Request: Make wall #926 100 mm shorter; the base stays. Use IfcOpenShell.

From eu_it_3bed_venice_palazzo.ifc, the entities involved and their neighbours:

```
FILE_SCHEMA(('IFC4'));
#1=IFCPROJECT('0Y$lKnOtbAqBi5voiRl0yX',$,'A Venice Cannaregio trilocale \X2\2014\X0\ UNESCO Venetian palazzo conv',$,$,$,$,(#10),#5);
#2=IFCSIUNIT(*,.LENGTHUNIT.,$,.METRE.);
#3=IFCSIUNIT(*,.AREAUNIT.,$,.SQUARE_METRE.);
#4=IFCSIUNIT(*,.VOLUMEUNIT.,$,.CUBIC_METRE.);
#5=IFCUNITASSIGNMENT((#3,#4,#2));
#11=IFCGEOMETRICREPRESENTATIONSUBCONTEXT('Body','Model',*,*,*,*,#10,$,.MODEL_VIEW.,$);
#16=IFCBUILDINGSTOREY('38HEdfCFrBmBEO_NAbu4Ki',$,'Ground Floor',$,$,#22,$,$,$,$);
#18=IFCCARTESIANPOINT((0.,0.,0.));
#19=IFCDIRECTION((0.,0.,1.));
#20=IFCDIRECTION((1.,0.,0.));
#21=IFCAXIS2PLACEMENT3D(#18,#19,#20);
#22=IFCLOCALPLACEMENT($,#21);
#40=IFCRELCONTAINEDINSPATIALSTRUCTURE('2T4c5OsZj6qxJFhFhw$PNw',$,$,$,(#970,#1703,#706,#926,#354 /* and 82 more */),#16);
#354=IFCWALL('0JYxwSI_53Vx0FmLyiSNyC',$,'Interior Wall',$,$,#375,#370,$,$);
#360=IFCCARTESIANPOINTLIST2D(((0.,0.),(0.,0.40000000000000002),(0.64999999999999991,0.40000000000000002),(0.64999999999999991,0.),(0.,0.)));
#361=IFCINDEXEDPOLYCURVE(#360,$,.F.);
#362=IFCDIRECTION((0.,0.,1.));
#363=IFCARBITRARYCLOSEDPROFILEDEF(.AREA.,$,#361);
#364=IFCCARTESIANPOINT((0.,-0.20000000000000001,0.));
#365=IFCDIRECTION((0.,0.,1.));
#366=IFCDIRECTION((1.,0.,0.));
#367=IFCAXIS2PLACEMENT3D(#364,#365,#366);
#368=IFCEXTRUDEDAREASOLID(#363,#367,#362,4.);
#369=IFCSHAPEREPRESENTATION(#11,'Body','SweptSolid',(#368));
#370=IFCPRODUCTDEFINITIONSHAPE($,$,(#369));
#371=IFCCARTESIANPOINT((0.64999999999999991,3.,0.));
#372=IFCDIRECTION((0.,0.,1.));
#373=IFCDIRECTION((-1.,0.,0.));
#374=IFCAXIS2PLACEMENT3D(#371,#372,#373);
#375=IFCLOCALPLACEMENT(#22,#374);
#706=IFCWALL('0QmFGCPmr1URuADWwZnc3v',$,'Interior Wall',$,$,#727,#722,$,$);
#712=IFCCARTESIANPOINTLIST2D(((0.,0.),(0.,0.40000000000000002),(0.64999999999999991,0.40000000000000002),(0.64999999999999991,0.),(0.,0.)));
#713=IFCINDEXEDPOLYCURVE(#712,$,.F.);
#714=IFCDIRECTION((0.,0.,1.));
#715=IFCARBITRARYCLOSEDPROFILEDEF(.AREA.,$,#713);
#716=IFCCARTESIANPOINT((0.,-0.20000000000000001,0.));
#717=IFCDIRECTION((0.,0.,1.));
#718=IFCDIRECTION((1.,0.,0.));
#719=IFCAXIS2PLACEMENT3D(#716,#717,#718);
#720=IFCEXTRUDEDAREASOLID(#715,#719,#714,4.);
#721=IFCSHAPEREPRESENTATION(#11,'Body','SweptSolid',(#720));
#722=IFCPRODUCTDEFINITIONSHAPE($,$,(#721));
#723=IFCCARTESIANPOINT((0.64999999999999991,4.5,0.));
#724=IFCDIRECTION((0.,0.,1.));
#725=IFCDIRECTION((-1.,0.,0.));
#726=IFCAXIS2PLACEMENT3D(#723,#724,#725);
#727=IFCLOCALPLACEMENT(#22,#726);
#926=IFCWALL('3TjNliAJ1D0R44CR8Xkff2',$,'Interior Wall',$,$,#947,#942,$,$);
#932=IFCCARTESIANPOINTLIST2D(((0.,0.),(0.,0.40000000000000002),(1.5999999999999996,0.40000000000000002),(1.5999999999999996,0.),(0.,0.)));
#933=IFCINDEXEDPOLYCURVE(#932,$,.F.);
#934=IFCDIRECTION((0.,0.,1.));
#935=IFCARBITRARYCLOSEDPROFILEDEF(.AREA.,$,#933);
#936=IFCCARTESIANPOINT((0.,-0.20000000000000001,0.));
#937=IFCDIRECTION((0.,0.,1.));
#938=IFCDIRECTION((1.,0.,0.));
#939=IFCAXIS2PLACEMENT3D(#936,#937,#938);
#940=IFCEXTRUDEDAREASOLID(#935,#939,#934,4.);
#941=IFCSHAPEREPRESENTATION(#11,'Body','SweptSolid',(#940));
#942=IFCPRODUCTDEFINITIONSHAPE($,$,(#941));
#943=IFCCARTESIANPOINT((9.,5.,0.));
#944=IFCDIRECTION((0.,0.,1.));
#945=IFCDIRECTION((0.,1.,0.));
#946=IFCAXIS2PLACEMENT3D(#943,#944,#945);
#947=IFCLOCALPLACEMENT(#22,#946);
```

```python
import ifcopenshell
import ifcopenshell.geom
import ifcopenshell.util.representation
import ifcopenshell.util.shape
import ifcopenshell.util.unit

model = ifcopenshell.open("eu_it_3bed_venice_palazzo.ifc")
unit_scale = ifcopenshell.util.unit.calculate_unit_scale(model)
settings = ifcopenshell.geom.settings()


def volume(element):
    """Net volume in cubic metres, openings subtracted."""
    shape = ifcopenshell.geom.create_shape(settings, element)
    return ifcopenshell.util.shape.get_volume(shape.geometry)


wall = model.by_guid("3TjNliAJ1D0R44CR8Xkff2")
before = volume(wall)

body = ifcopenshell.util.representation.get_representation(wall, "Model", "Body")
solid = body.Items[0]
old_height = solid.Depth
solid.Depth -= 0.1 / unit_scale
after = volume(wall)

print(f"height {old_height:g} -> {solid.Depth:g}, volume {before:.3f} -> {after:.3f} m3")

model.write("eu_it_3bed_venice_palazzo_v2.ifc")
```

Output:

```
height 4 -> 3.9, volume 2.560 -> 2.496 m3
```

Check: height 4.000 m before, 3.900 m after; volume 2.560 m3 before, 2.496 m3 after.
